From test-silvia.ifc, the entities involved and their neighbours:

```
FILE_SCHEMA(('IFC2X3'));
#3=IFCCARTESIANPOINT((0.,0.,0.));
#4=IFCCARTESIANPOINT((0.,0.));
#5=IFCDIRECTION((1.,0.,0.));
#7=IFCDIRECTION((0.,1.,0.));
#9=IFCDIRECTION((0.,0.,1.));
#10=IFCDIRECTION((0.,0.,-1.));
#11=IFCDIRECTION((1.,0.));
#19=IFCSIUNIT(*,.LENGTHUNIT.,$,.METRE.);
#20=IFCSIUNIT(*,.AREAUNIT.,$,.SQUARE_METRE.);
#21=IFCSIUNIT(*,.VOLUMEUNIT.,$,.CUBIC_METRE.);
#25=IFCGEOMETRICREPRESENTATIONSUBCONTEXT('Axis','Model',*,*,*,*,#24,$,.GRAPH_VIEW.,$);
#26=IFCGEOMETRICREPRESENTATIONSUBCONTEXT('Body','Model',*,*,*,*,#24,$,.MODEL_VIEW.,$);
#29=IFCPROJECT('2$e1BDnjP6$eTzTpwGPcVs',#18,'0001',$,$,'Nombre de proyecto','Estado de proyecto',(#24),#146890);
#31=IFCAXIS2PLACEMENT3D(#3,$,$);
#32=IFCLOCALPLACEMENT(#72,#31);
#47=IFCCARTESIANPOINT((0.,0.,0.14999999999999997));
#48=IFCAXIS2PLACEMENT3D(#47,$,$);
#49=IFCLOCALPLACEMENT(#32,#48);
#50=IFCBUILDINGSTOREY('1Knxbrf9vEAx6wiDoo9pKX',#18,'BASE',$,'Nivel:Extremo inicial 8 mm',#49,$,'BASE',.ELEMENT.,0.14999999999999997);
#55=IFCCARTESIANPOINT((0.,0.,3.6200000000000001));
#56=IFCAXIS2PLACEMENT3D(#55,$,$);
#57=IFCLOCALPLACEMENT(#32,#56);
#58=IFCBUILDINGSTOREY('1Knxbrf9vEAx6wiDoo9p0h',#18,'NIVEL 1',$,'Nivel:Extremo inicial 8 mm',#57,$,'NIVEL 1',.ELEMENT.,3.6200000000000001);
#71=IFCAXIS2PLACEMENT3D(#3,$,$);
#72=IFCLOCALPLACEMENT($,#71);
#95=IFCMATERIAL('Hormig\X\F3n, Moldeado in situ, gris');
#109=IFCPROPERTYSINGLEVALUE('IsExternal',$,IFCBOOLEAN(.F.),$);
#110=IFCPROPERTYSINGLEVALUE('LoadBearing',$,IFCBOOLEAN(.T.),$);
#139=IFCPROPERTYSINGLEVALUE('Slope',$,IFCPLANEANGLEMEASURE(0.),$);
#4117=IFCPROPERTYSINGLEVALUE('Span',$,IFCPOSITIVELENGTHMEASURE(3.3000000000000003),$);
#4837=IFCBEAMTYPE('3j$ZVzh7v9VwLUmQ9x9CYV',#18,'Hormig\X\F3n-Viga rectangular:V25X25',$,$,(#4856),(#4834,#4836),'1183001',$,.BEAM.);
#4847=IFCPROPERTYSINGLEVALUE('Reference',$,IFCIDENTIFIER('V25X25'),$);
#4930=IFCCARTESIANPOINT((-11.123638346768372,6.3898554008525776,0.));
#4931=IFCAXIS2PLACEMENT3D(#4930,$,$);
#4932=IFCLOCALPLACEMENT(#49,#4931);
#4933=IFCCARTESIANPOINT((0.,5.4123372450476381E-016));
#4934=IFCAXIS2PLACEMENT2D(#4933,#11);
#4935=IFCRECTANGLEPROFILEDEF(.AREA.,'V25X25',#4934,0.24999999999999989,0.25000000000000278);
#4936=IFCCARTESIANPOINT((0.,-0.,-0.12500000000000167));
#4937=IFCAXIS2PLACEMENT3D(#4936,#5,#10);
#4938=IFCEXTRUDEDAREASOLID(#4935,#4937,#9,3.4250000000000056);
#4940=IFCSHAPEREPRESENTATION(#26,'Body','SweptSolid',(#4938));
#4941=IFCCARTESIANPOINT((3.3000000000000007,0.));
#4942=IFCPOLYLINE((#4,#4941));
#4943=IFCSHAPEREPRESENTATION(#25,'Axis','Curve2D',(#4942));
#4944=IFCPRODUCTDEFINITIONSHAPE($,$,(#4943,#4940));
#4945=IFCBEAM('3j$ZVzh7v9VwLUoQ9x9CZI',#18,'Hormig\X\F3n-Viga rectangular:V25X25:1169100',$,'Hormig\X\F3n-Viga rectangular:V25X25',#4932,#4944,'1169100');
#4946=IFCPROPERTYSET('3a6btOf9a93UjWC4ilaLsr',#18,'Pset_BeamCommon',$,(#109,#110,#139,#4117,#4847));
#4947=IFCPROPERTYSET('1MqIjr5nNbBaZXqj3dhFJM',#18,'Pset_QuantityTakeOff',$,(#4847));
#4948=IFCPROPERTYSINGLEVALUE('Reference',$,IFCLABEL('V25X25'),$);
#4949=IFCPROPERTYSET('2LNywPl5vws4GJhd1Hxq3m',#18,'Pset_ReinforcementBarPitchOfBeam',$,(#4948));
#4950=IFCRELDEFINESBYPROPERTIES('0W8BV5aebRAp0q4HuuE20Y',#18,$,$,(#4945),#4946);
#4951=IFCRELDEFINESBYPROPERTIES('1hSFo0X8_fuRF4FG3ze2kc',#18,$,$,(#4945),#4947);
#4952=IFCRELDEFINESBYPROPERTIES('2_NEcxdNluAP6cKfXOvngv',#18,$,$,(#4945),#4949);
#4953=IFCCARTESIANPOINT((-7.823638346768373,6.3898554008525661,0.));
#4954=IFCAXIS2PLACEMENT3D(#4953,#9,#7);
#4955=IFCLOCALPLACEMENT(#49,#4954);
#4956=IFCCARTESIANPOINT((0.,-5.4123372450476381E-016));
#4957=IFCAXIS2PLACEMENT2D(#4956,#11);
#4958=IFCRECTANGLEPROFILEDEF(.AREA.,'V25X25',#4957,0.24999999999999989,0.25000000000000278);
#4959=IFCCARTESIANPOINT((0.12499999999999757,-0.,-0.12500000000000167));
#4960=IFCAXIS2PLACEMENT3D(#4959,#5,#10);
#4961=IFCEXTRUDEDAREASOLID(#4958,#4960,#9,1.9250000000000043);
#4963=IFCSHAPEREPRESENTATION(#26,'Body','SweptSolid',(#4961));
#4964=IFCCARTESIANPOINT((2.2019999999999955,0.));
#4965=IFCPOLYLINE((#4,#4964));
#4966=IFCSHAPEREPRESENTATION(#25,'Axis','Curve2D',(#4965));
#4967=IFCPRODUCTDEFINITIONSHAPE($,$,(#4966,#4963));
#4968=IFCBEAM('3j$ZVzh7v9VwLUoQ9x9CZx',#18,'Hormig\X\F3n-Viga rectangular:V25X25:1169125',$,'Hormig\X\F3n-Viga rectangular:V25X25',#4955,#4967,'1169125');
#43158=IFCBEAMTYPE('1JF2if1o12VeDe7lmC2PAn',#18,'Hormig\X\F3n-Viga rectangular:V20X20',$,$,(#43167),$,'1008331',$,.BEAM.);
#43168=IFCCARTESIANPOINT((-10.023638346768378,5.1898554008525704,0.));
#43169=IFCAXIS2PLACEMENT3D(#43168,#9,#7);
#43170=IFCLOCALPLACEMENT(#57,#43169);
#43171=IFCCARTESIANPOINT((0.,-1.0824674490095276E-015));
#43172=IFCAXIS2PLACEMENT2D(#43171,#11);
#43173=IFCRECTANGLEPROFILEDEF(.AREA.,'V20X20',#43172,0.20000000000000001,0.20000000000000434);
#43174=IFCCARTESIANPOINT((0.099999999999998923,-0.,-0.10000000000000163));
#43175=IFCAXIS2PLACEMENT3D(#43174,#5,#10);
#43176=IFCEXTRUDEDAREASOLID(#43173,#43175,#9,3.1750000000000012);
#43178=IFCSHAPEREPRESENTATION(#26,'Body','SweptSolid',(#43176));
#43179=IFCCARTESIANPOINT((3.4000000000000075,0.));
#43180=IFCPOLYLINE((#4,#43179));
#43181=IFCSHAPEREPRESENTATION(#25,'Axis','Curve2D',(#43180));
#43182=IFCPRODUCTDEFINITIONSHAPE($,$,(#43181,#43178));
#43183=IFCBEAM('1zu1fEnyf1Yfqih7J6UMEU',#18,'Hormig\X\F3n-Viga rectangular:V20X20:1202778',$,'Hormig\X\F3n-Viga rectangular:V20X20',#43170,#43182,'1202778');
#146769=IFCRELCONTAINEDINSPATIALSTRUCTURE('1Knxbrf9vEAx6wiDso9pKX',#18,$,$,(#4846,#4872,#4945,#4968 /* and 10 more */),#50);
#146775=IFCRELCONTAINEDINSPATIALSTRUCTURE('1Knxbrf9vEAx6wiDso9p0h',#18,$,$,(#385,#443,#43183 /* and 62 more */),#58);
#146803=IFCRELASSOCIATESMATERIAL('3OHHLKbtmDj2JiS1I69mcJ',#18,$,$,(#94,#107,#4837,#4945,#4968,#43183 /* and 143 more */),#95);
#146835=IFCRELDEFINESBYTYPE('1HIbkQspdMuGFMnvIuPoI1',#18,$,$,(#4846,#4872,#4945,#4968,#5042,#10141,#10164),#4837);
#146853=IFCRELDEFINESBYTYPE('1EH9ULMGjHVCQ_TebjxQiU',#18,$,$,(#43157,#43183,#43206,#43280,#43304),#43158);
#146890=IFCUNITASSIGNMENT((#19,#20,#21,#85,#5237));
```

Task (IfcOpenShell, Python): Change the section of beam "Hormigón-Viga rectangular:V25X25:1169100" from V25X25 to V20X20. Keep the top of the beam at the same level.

```python
import ifcopenshell
import ifcopenshell.api.pset
import ifcopenshell.api.type
import ifcopenshell.util.element
import ifcopenshell.util.representation

model = ifcopenshell.open("test-silvia.ifc")

member = model.by_guid("3j$ZVzh7v9VwLUoQ9x9CZI")
source = next(p for p in model.by_type("IfcRectangleProfileDef") if p.ProfileName == "V20X20")

body = ifcopenshell.util.representation.get_representation(member, "Model", "Body")
solid = body.Items[0]
old_profile = solid.SweptArea

# Copy the section's sizes but keep this member's own profile position.
profile = ifcopenshell.util.element.copy(model, source)
# Profiles are centred, so shift by half the change in depth to hold the top.
shift = (old_profile.XDim - profile.XDim) / 2
x, y = old_profile.Position.Location.Coordinates
up = (-1.0, 0.0)  # upwards, in the solid's own plane
location = model.createIfcCartesianPoint((x + up[0] * shift, y + up[1] * shift))
profile.Position = model.createIfcAxis2Placement2D(location, old_profile.Position.RefDirection)
solid.SweptArea = profile
if not model.get_total_inverses(old_profile):
    ifcopenshell.util.element.remove_deep2(model, old_profile)

new_type = model.by_id(43158)
ifcopenshell.api.type.assign_type(
    model, related_objects=[member], relating_type=new_type, should_map_representations=False
)
member.Name = member.Name.replace("V25X25", "V20X20")
member.ObjectType = "Hormigón-Viga rectangular:V20X20"
pset = model.by_id(ifcopenshell.util.element.get_pset(member, "Pset_BeamCommon", should_inherit=False)["id"])
ifcopenshell.api.pset.edit_pset(model, pset=pset, properties={"Reference": "V20X20"})
pset = model.by_id(ifcopenshell.util.element.get_pset(member, "Pset_QuantityTakeOff", should_inherit=False)["id"])
ifcopenshell.api.pset.edit_pset(model, pset=pset, properties={"Reference": "V20X20"})
pset = model.by_id(ifcopenshell.util.element.get_pset(member, "Pset_ReinforcementBarPitchOfBeam", should_inherit=False)["id"])
ifcopenshell.api.pset.edit_pset(model, pset=pset, properties={"Reference": "V20X20"})

print(solid.SweptArea)

model.write("test-silvia_rev.ifc")
```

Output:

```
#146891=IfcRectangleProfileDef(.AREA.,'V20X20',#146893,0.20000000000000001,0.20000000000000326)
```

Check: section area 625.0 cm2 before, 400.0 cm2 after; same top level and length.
